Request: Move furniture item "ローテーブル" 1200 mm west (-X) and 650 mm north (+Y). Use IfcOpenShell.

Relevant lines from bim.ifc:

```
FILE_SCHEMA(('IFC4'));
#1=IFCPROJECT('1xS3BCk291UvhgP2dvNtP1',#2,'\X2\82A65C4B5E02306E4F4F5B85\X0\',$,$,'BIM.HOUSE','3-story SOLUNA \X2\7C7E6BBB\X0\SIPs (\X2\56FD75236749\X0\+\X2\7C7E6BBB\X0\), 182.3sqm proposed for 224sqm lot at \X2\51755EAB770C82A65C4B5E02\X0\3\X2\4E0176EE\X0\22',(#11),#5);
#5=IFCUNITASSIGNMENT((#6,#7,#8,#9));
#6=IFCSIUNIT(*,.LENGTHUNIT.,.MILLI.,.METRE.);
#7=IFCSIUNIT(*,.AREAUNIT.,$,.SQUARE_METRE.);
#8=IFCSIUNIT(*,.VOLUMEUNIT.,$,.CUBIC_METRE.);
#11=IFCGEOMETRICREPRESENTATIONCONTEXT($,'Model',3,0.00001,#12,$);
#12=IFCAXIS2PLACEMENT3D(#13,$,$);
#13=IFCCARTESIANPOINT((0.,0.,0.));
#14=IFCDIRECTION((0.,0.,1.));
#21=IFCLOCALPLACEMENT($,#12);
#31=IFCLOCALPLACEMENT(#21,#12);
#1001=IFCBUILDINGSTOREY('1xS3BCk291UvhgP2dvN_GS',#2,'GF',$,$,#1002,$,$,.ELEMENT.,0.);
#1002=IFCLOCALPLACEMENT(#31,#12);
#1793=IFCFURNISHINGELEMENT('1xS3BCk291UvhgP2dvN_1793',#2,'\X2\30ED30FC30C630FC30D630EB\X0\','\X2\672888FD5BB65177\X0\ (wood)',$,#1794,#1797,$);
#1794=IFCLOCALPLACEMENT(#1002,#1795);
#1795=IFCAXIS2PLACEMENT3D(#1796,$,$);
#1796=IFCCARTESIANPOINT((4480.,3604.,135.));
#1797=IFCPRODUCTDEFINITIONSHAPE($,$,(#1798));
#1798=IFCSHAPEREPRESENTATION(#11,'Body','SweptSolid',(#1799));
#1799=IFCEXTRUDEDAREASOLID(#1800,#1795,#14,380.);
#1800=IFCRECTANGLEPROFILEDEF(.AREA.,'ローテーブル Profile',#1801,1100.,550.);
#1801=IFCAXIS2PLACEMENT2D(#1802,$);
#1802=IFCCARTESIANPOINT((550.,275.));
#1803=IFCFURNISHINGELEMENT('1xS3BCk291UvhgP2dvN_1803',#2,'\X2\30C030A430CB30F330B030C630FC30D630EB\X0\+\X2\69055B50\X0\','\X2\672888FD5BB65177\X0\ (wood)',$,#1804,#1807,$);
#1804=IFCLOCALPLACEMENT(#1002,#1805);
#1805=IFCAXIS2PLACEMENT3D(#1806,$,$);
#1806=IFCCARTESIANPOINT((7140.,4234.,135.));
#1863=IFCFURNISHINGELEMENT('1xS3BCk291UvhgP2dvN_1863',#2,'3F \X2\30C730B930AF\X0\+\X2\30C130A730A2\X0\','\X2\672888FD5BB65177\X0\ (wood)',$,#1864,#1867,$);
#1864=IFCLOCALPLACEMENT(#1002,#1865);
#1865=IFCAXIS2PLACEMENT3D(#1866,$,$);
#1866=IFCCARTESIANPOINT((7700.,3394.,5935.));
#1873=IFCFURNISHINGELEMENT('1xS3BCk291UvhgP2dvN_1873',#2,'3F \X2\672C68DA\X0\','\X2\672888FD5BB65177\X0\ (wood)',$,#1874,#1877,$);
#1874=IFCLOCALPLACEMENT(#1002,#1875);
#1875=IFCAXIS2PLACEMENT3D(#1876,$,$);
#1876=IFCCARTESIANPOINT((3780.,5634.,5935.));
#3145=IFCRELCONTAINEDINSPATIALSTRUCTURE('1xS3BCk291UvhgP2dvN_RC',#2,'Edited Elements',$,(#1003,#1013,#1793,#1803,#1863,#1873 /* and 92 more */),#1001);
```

```python
import ifcopenshell
import ifcopenshell.api.geometry
import ifcopenshell.util.placement

model = ifcopenshell.open("bim.ifc")

item = model.by_id(1793)
matrix = ifcopenshell.util.placement.get_local_placement(item.ObjectPlacement)
matrix[0, 3] -= 1200.0
matrix[1, 3] += 650.0
ifcopenshell.api.geometry.edit_object_placement(model, product=item, matrix=matrix, is_si=False)

print(ifcopenshell.util.placement.get_local_placement(item.ObjectPlacement).round(3) + 0.0)

model.write("bim_edited.ifc")
```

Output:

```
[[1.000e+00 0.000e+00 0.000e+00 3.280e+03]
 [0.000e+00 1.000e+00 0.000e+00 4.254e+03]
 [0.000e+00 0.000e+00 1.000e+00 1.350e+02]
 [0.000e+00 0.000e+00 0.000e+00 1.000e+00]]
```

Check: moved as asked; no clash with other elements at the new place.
